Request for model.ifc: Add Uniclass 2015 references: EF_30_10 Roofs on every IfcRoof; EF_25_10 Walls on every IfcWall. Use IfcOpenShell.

First a look at what the model holds.

```python
import ifcopenshell

model = ifcopenshell.open("model.ifc")
print(model.schema)
print("classifications:", [c.Name for c in model.by_type("IfcClassification")])
for ifc_class in ("IfcDoor", "IfcRoof", "IfcStair", "IfcWall", "IfcWindow"):
    print(ifc_class, len(model.by_type(ifc_class)))
```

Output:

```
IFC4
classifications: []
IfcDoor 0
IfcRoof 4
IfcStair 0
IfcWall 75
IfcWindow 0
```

```python
import ifcopenshell
import ifcopenshell.api.classification

model = ifcopenshell.open("model.ifc")

system = ifcopenshell.api.classification.add_classification(model, classification="Uniclass 2015")

codes = {
    "IfcRoof": ("EF_30_10", "Roofs"),
    "IfcWall": ("EF_25_10", "Walls"),
}
for ifc_class, (code, name) in codes.items():
    products = model.by_type(ifc_class)
    ifcopenshell.api.classification.add_reference(
        model, products=products, classification=system, identification=code, name=name
    )
    print(code, len(products))

model.write("model-out.ifc")
```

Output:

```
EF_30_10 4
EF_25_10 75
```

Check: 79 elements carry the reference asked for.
